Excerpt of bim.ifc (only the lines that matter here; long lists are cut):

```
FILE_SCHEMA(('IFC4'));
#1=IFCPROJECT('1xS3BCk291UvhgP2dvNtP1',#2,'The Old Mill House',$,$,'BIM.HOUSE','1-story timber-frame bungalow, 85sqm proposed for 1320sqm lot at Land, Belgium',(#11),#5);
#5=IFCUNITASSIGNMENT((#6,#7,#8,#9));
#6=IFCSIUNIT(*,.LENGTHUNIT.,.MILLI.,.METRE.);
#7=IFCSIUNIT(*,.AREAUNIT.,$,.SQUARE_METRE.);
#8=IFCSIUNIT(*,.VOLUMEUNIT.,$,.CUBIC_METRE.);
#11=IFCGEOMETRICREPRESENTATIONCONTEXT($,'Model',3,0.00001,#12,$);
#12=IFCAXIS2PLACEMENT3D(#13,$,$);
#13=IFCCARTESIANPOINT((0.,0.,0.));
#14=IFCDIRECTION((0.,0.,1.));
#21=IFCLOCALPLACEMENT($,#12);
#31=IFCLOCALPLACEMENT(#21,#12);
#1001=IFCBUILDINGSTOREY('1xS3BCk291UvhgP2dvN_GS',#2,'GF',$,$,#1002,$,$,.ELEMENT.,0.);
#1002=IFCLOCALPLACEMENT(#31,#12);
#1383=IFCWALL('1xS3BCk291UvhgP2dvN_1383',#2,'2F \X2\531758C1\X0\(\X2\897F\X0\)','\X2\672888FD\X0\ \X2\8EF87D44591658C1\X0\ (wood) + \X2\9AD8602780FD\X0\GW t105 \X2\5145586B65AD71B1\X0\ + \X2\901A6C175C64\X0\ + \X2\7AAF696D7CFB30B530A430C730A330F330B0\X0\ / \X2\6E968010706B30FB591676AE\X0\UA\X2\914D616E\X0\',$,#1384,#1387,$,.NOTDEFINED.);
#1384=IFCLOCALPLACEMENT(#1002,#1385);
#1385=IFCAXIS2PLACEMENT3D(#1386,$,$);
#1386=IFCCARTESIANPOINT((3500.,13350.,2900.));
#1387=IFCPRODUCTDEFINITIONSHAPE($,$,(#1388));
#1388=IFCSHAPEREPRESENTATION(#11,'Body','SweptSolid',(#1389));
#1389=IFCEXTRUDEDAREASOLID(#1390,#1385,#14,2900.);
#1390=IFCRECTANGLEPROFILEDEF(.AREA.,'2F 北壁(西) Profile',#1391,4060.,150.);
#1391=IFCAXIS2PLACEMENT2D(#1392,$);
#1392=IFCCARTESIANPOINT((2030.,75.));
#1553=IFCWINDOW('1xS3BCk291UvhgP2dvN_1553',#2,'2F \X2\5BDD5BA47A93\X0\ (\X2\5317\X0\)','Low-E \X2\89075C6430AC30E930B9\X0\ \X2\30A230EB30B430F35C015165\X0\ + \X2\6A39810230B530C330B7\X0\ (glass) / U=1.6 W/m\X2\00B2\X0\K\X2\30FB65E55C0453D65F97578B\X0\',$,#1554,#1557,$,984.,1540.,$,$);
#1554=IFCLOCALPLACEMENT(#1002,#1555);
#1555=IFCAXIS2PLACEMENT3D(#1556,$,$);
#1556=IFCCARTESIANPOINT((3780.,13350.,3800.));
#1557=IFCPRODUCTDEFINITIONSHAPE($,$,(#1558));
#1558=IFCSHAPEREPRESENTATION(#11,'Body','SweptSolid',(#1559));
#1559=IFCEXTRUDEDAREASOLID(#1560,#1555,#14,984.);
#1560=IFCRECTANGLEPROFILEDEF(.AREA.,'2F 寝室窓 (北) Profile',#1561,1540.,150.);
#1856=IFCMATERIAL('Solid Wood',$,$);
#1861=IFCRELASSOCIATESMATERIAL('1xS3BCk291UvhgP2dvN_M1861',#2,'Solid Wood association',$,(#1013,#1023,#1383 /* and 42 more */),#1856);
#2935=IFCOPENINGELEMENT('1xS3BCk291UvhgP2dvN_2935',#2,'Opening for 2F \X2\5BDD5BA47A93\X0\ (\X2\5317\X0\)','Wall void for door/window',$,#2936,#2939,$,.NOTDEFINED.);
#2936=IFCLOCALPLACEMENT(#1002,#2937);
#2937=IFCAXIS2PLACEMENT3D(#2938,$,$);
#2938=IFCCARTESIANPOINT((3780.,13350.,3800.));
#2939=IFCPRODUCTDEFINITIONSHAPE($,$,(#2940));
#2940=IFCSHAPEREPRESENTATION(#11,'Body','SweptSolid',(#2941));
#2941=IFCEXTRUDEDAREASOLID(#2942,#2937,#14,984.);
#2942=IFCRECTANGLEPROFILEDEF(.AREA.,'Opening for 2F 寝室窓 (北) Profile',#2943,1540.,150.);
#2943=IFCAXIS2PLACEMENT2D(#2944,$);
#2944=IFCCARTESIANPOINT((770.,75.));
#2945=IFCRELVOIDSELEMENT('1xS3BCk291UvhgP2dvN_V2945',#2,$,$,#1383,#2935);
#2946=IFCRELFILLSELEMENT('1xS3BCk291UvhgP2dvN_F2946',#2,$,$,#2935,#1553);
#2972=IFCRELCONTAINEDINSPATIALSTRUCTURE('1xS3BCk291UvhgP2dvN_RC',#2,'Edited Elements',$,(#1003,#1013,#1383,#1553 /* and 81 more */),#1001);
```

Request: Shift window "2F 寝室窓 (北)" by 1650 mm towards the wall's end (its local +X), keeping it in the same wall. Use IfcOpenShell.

```python
import ifcopenshell
import ifcopenshell.api.geometry
import ifcopenshell.util.placement

model = ifcopenshell.open("bim.ifc")

window = model.by_guid("1xS3BCk291UvhgP2dvN_1553")
opening = window.FillsVoids[0].RelatingOpeningElement
wall = opening.VoidsElements[0].RelatingBuildingElement

wall_matrix = ifcopenshell.util.placement.get_local_placement(wall.ObjectPlacement)
shift = wall_matrix[:3, 0] * 1650.0
before = ifcopenshell.util.placement.get_local_placement(window.ObjectPlacement)[:3, 3].copy()

# The window is not placed relative to its opening, so move both.
for product in (opening, window):
    matrix = ifcopenshell.util.placement.get_local_placement(product.ObjectPlacement)
    matrix[:3, 3] += shift
    ifcopenshell.api.geometry.edit_object_placement(model, product=product, matrix=matrix, is_si=False)

after = ifcopenshell.util.placement.get_local_placement(window.ObjectPlacement)[:3, 3]
print("window moved by", (after - before).round(3) + 0.0)

model.write("bim-out.ifc")
```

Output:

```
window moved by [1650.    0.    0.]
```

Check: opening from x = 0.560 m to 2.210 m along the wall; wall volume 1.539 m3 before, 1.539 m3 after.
